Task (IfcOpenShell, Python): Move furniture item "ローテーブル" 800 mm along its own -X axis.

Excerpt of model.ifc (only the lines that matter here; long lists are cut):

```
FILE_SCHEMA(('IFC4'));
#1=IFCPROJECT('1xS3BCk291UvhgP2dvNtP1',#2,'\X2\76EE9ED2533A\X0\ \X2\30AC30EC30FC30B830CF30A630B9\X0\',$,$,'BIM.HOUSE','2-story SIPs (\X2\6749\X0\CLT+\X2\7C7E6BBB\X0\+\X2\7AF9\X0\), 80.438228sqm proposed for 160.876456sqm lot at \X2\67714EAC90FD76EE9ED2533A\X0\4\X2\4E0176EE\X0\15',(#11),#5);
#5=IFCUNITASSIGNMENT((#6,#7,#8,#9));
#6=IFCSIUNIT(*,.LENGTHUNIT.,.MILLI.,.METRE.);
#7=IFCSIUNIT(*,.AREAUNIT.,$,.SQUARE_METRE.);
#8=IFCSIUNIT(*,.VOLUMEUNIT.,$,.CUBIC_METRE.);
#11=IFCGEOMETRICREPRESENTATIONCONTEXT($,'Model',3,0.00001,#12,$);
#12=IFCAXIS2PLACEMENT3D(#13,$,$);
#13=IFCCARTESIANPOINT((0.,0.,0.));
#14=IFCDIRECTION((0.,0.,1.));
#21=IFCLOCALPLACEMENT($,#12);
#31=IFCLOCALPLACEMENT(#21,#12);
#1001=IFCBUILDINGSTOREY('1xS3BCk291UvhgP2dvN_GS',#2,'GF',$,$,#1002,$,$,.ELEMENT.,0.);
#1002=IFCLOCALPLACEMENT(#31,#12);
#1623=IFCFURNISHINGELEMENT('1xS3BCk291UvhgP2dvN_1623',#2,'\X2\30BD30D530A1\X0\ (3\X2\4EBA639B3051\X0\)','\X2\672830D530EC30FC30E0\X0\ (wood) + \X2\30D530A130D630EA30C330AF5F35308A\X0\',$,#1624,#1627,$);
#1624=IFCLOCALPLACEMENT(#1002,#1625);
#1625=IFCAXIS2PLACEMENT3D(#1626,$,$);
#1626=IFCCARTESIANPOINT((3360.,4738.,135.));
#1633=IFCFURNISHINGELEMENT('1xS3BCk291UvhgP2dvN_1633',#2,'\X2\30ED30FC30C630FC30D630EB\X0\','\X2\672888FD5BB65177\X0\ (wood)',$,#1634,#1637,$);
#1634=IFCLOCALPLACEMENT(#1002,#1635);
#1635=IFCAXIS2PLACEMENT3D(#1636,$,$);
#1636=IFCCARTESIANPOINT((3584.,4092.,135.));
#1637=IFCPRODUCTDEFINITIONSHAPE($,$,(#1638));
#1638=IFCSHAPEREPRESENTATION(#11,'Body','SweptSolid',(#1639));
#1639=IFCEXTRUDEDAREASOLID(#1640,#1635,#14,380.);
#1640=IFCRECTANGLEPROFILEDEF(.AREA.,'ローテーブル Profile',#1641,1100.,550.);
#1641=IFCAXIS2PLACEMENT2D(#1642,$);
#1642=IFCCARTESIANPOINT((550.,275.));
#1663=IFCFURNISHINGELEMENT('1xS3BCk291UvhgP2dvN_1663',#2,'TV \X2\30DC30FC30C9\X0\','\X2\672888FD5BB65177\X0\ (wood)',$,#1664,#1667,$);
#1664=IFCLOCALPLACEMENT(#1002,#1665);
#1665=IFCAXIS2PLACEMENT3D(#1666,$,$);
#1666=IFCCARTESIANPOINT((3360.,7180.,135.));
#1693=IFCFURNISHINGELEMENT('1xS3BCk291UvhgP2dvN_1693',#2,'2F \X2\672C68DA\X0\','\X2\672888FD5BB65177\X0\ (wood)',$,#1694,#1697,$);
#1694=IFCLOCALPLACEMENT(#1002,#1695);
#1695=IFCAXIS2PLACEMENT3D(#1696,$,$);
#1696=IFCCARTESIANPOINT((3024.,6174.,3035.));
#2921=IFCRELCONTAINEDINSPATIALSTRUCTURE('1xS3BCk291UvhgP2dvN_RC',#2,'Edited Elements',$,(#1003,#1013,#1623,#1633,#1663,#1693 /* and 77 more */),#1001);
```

```python
import ifcopenshell
import ifcopenshell.api.geometry
import ifcopenshell.util.placement
import ifcopenshell.util.unit

model = ifcopenshell.open("model.ifc")
unit_scale = ifcopenshell.util.unit.calculate_unit_scale(model)

item = model.by_id(1633)
matrix = ifcopenshell.util.placement.get_local_placement(item.ObjectPlacement)
matrix[:3, 3] -= matrix[:3, 0] * 0.8 / unit_scale
ifcopenshell.api.geometry.edit_object_placement(model, product=item, matrix=matrix, is_si=False)

print(ifcopenshell.util.placement.get_local_placement(item.ObjectPlacement).round(3) + 0.0)

model.write("model_edited.ifc")
```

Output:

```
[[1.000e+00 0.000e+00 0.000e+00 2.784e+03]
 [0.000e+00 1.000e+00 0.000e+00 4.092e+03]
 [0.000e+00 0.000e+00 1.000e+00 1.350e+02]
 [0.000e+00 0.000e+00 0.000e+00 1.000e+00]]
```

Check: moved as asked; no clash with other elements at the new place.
